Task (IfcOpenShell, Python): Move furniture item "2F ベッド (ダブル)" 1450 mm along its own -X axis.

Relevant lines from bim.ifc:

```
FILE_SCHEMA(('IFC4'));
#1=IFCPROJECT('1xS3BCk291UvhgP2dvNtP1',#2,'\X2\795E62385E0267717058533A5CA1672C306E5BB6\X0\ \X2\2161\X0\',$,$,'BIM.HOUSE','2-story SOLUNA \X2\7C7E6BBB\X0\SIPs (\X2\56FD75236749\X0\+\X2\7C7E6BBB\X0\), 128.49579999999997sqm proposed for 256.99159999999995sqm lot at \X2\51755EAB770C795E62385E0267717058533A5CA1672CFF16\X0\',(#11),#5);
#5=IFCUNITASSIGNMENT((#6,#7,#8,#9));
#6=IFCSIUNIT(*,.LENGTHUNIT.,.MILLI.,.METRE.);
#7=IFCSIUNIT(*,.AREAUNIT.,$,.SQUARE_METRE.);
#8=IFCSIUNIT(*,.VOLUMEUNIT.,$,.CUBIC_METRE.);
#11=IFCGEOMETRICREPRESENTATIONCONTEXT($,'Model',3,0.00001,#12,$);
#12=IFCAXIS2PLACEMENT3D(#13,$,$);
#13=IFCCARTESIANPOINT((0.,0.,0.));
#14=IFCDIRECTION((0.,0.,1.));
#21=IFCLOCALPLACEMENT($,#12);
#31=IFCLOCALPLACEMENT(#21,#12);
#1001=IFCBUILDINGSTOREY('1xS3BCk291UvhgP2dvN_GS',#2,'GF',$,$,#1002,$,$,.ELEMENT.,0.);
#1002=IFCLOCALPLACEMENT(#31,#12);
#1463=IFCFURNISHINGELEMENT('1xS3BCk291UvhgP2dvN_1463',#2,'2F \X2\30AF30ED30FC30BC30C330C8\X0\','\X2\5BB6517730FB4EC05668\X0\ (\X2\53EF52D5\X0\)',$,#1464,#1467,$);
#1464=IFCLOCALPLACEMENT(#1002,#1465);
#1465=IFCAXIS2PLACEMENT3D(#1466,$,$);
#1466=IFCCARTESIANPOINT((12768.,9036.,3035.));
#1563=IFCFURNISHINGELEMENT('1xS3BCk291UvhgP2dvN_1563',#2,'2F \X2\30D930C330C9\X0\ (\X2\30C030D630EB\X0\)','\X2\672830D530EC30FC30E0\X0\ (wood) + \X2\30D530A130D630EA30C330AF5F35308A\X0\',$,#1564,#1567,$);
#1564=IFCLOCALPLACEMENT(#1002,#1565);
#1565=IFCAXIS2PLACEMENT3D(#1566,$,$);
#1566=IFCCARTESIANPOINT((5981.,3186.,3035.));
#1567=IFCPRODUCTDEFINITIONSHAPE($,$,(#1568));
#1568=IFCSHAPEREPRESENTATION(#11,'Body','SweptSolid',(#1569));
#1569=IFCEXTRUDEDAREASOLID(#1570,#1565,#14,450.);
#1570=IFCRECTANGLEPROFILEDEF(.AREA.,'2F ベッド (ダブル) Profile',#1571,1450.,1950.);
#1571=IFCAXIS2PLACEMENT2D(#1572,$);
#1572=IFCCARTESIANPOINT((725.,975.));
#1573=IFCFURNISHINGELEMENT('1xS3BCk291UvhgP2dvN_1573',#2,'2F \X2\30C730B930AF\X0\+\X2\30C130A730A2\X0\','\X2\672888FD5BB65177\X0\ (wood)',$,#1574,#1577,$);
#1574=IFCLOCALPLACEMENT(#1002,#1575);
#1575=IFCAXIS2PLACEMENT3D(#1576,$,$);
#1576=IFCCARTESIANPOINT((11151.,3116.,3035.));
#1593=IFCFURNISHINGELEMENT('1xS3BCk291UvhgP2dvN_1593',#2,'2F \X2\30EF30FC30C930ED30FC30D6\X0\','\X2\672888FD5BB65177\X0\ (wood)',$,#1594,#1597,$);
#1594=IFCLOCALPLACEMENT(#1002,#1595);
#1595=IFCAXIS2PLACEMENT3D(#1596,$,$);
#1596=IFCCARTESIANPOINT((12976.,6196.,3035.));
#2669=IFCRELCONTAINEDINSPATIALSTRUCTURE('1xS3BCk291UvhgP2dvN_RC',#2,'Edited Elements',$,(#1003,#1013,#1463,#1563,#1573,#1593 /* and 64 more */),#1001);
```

```python
import ifcopenshell
import ifcopenshell.api.geometry
import ifcopenshell.util.placement

model = ifcopenshell.open("bim.ifc")

item = model.by_guid("1xS3BCk291UvhgP2dvN_1563")
matrix = ifcopenshell.util.placement.get_local_placement(item.ObjectPlacement)
matrix[:3, 3] -= matrix[:3, 0] * 1450.0
ifcopenshell.api.geometry.edit_object_placement(model, product=item, matrix=matrix, is_si=False)

print(ifcopenshell.util.placement.get_local_placement(item.ObjectPlacement).round(3) + 0.0)

model.write("bim_v2.ifc")
```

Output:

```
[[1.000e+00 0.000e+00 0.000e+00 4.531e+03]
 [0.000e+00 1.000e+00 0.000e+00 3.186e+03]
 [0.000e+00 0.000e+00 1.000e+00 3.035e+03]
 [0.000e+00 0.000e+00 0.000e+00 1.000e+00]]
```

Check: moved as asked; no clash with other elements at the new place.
